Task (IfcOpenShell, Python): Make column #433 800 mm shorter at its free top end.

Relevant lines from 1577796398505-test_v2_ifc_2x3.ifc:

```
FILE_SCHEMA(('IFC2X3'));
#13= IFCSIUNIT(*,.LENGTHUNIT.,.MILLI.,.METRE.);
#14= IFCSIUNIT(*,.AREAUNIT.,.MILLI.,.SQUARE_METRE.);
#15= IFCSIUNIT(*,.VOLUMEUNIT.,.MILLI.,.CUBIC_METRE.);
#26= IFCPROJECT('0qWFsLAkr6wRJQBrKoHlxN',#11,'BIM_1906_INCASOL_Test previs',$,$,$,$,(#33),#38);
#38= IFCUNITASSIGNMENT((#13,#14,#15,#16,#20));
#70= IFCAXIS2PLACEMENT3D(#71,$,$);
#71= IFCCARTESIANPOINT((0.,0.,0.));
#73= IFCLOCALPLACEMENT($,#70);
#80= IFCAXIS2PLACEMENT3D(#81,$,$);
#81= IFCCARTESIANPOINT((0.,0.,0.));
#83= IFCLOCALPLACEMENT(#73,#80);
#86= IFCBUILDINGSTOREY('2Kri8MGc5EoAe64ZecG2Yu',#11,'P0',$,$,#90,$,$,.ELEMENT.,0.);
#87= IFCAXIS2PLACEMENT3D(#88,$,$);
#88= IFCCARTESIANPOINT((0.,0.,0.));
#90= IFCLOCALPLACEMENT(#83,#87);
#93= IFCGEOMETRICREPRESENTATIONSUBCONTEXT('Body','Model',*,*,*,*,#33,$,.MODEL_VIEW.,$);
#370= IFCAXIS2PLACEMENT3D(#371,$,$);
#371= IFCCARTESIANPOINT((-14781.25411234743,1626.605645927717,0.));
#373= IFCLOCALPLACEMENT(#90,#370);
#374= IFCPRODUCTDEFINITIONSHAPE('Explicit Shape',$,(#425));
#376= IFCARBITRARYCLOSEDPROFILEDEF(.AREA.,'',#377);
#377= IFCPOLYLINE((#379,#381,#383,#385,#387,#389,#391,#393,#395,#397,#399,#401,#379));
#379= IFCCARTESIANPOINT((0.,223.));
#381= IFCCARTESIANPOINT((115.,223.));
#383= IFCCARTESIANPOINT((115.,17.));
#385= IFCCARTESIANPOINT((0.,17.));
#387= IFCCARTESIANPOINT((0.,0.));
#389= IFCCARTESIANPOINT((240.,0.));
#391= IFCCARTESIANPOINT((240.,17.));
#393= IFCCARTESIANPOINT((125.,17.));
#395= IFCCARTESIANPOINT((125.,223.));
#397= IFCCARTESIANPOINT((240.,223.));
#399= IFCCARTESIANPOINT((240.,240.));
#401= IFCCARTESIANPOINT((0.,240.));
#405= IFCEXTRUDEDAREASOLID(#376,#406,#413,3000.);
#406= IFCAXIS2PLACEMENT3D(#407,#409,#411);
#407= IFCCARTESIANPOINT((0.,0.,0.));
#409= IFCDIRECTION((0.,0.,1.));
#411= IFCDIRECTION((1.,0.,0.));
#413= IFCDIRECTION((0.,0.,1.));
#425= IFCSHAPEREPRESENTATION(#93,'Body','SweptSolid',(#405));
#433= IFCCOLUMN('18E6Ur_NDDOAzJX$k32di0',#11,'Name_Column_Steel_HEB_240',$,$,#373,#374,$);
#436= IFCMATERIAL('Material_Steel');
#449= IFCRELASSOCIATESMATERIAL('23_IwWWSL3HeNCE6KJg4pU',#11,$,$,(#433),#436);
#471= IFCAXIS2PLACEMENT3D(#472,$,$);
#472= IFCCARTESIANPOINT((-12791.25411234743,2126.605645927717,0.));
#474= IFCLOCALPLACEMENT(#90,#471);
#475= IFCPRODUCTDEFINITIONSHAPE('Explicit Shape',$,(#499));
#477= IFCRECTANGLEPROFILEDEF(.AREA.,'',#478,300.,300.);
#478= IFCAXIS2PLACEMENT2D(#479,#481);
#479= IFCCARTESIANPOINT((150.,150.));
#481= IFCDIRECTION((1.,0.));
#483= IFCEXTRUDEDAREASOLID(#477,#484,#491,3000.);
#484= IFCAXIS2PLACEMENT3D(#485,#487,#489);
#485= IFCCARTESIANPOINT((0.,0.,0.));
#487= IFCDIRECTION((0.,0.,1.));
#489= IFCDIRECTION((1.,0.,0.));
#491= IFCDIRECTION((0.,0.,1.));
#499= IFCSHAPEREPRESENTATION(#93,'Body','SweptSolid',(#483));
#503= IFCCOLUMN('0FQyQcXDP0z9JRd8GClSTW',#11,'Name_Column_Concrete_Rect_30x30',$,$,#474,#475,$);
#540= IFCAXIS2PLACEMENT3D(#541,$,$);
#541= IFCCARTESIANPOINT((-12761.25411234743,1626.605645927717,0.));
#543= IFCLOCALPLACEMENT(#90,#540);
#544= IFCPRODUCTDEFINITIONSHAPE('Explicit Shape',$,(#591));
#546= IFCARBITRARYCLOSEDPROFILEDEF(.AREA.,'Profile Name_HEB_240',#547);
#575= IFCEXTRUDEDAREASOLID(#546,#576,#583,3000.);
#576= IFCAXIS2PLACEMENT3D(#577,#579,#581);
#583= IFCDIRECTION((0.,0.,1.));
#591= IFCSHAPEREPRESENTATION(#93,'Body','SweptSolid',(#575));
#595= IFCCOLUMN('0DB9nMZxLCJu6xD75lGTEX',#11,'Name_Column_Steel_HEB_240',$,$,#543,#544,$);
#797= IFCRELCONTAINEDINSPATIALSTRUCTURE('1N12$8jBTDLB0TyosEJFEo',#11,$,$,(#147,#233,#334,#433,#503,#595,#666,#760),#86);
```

```python
import ifcopenshell
import ifcopenshell.util.representation

model = ifcopenshell.open("1577796398505-test_v2_ifc_2x3.ifc")

member = model.by_id(433)
change = -800.0

# The extrusion runs towards the end named, so only its depth changes.
body = ifcopenshell.util.representation.get_representation(member, "Model", "Body")
solid = body.Items[0]
old_length = solid.Depth
solid.Depth += change

print(f"length {old_length:g} -> {solid.Depth:g}")

model.write("1577796398505-test_v2_ifc_2x3-out.ifc")
```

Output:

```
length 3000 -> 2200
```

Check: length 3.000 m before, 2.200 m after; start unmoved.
